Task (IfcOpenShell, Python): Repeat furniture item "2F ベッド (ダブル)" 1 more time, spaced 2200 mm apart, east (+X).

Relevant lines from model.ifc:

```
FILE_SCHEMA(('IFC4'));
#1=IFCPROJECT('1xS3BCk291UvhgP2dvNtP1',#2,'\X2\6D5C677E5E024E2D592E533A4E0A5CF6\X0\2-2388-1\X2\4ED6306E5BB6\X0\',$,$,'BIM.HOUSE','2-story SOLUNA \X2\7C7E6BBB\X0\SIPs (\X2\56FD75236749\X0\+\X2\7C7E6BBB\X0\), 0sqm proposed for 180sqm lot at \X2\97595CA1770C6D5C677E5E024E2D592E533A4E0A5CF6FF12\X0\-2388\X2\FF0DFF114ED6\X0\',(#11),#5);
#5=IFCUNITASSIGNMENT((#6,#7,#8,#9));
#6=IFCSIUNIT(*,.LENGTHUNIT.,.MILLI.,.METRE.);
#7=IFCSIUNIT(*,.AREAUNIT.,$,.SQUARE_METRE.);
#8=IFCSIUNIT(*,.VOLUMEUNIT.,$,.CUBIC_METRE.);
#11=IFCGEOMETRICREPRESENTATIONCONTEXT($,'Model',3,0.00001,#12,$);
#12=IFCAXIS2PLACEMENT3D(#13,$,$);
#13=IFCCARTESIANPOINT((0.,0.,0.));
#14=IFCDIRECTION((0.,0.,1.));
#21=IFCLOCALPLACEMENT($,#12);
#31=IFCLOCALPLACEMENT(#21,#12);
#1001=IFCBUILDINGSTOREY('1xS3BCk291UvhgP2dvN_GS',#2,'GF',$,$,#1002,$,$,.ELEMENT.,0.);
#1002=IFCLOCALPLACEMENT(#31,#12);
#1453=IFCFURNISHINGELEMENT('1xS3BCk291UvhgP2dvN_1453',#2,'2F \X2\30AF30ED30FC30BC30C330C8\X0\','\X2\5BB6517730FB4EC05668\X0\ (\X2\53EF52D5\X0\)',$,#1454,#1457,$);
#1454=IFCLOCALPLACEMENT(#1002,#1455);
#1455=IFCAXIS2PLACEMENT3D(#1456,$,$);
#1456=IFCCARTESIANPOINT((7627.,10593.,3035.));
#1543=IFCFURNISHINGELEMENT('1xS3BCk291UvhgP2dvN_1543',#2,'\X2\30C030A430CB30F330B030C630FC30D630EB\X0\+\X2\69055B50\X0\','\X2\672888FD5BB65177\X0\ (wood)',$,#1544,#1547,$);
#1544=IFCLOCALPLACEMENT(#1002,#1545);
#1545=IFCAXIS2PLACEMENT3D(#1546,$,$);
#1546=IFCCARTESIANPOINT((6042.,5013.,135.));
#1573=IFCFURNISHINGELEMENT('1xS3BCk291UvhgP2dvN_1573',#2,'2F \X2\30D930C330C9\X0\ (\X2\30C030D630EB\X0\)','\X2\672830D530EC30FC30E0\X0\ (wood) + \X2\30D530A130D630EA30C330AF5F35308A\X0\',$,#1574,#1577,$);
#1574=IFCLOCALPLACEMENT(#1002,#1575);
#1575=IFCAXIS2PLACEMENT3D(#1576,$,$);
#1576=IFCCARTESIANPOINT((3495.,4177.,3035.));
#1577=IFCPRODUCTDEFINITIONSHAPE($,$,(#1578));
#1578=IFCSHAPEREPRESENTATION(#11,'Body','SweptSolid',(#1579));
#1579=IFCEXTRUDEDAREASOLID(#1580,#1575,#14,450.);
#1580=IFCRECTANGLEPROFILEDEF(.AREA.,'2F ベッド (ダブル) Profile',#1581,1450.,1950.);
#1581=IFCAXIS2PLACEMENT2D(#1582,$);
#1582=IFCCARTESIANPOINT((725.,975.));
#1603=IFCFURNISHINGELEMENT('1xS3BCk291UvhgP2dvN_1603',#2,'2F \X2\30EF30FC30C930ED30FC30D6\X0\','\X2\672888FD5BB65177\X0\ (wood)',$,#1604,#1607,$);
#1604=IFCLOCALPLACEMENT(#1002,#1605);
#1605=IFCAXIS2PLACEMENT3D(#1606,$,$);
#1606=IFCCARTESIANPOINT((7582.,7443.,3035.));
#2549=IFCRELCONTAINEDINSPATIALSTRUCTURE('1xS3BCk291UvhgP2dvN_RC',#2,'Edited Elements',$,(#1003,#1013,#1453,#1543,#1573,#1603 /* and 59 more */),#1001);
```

```python
import numpy as np
import ifcopenshell
import ifcopenshell.api.geometry
import ifcopenshell.api.root
import ifcopenshell.util.element
import ifcopenshell.util.placement

model = ifcopenshell.open("model.ifc")


def reuse_history(source, copy):
    """copy_class also copies each property set's owner history, people and application; keep the originals."""
    for rel in copy.IsDefinedBy:
        if rel.is_a("IfcRelDefinesByProperties") and (history := rel.RelatingPropertyDefinition.OwnerHistory):
            rel.RelatingPropertyDefinition.OwnerHistory = source.OwnerHistory
            ifcopenshell.util.element.remove_deep2(model, history)


source = model.by_guid("1xS3BCk291UvhgP2dvN_1573")
base = ifcopenshell.util.placement.get_local_placement(source.ObjectPlacement)
step = np.array([1.0, 0.0, 0.0]) * 2200.0

for i in range(1, 2):
    copy = ifcopenshell.api.root.copy_class(model, product=source)
    copy.Representation = ifcopenshell.util.element.copy_deep(
        model, source.Representation, exclude=["IfcGeometricRepresentationContext", "IfcRepresentationMap"]
    )
    reuse_history(source, copy)
    matrix = base.copy()
    matrix[:3, 3] += i * step
    print("added at", matrix[:3, 3].round(3) + 0.0)
    ifcopenshell.api.geometry.edit_object_placement(model, product=copy, matrix=matrix, is_si=False)

model.write("model_v2.ifc")
```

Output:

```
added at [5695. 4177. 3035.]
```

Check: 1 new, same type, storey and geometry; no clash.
